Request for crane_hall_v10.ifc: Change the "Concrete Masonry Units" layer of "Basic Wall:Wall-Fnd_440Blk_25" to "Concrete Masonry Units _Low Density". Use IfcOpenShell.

First a look at what the model holds.

```python
import ifcopenshell
import ifcopenshell.util.element

model = ifcopenshell.open("crane_hall_v10.ifc")
print(model.schema)
for layer_set in model.by_type("IfcMaterialLayerSet"):
    if layer_set.LayerSetName == "Basic Wall:Wall-Fnd_440Blk_25":
        for layer in layer_set.MaterialLayers:
            print(layer.id(), layer.Material and layer.Material.Name, layer.LayerThickness, sep=" | ")
        print(len(ifcopenshell.util.element.get_elements_by_material(model, layer_set)), "elements and types use it")
print(sorted(m.Name for m in model.by_type("IfcMaterial") if m.Name)[:60])
```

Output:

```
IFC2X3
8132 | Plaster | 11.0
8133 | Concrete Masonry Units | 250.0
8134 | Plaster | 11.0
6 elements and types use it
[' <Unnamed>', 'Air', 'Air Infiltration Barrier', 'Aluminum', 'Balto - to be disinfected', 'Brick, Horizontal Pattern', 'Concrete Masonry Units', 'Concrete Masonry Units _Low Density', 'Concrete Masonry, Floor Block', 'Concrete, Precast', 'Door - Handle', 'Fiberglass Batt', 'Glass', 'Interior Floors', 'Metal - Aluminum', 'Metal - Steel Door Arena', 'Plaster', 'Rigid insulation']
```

```python
import ifcopenshell
import ifcopenshell.api.material

model = ifcopenshell.open("crane_hall_v10.ifc")

layer_set = next(s for s in model.by_type("IfcMaterialLayerSet") if s.LayerSetName == "Basic Wall:Wall-Fnd_440Blk_25")
layer = next(l for l in layer_set.MaterialLayers if l.Material and l.Material.Name == "Concrete Masonry Units")
material = next(m for m in model.by_type("IfcMaterial") if m.Name == "Concrete Masonry Units _Low Density")

# Point this one layer at the other material; renaming the old one would change it everywhere.
ifcopenshell.api.material.edit_layer(model, layer=layer, attributes={}, material=material)

print([l.Material.Name if l.Material else None for l in layer_set.MaterialLayers])

model.write("crane_hall_v10_edited.ifc")
```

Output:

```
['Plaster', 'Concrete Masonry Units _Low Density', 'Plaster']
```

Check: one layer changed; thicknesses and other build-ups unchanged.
